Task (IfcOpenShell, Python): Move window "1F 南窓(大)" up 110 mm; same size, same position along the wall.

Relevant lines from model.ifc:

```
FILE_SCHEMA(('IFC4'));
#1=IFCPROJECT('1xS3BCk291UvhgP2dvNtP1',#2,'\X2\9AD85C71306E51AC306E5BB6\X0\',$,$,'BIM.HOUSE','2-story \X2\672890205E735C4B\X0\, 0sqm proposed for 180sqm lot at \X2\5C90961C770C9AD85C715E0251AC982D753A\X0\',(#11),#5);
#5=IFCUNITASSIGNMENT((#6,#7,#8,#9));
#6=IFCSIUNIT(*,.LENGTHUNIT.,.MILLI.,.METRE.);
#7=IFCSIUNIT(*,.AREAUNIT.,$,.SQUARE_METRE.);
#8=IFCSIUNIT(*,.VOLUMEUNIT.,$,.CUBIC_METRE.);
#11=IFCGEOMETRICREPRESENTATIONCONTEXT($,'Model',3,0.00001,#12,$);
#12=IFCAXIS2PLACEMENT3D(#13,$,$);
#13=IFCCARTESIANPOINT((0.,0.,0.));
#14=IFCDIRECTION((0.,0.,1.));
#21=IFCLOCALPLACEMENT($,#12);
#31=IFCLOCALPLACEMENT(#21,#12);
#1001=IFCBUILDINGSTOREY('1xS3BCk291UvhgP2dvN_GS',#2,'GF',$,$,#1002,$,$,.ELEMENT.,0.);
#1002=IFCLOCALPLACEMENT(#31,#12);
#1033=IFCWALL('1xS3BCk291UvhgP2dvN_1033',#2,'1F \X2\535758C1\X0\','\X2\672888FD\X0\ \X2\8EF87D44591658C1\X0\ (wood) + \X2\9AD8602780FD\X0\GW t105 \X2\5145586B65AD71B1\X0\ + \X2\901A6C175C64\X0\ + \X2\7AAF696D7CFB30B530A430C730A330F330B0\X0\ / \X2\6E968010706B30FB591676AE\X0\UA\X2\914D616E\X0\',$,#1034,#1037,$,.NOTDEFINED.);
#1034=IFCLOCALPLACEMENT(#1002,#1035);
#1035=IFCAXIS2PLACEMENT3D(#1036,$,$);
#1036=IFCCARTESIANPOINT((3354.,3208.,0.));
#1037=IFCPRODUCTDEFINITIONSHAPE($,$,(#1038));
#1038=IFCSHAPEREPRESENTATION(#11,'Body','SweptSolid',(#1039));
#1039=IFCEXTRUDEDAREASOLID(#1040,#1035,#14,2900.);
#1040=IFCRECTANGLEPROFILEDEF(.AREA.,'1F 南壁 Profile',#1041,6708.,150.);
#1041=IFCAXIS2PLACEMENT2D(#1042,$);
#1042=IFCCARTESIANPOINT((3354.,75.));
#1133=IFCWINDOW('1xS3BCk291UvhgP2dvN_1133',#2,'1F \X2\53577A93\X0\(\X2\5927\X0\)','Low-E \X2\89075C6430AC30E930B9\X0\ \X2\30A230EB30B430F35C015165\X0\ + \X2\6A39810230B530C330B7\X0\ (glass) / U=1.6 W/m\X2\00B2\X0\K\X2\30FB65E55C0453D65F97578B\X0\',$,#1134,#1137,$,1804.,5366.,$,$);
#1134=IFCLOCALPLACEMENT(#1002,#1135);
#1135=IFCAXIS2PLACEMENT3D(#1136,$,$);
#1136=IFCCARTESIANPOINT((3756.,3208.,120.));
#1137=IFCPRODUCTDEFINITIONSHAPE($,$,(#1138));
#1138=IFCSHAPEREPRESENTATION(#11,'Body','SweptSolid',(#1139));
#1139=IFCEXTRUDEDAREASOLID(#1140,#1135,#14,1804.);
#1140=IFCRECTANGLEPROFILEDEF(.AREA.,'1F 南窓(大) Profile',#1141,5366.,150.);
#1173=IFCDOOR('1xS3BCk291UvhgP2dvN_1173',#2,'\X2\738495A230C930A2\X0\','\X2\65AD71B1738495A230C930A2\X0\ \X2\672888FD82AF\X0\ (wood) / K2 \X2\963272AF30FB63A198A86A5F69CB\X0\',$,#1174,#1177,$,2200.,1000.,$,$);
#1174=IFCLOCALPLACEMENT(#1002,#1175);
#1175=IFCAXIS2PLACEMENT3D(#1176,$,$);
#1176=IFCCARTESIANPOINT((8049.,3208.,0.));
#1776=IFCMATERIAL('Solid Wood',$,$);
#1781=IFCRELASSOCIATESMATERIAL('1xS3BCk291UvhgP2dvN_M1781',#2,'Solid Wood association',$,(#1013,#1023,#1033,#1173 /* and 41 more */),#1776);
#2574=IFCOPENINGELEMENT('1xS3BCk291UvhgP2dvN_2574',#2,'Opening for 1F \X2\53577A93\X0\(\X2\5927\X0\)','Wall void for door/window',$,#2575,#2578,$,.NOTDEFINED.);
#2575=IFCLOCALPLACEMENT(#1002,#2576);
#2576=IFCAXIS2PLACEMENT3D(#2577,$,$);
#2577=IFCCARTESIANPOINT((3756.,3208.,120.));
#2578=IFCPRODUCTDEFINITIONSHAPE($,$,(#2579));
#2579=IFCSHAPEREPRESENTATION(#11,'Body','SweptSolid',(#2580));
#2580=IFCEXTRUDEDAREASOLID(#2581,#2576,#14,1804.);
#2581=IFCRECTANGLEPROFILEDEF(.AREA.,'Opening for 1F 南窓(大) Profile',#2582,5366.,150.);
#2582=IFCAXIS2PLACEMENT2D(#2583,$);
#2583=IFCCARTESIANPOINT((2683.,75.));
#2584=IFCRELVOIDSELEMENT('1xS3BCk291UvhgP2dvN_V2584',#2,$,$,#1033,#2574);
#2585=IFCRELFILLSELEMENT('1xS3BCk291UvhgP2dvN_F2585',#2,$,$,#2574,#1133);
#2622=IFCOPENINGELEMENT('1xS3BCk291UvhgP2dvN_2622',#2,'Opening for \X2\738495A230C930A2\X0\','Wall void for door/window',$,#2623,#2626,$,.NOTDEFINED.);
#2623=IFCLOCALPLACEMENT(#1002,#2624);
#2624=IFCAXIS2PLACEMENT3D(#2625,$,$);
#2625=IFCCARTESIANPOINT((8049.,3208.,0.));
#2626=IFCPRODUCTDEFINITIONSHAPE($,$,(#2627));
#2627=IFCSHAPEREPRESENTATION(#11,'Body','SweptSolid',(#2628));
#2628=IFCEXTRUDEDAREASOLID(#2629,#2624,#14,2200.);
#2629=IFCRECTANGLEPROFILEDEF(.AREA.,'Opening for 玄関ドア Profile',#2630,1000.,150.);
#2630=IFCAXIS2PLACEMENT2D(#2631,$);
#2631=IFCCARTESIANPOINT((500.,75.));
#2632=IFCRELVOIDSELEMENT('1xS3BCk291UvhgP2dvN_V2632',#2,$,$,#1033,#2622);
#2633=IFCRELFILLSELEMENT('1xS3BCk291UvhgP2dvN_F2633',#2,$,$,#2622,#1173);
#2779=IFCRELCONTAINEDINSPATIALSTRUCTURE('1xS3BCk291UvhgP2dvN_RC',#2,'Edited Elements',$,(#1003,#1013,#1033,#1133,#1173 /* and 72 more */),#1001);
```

```python
import numpy as np
import ifcopenshell
import ifcopenshell.api.geometry
import ifcopenshell.util.placement
import ifcopenshell.util.unit

model = ifcopenshell.open("model.ifc")
unit_scale = ifcopenshell.util.unit.calculate_unit_scale(model)

window = model.by_guid("1xS3BCk291UvhgP2dvN_1133")
opening = window.FillsVoids[0].RelatingOpeningElement
dz = 0.11 / unit_scale

shift = np.array([0.0, 0.0, dz])
# The window is not placed relative to its opening, so move both.
for product in (opening, window):
    matrix = ifcopenshell.util.placement.get_local_placement(product.ObjectPlacement)
    matrix[:3, 3] += shift
    ifcopenshell.api.geometry.edit_object_placement(model, product=product, matrix=matrix, is_si=False)

print(f"moved by {dz * unit_scale:+.3f} m")

model.write("model_edited.ifc")
```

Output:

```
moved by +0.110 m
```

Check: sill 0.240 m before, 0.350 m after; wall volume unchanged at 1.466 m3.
